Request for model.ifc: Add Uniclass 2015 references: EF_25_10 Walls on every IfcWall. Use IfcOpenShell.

First a look at what the model holds.

```python
import ifcopenshell

model = ifcopenshell.open("model.ifc")
print(model.schema)
print("classifications:", [c.Name for c in model.by_type("IfcClassification")])
for ifc_class in ("IfcDoor", "IfcRoof", "IfcStair", "IfcWall", "IfcWindow"):
    print(ifc_class, len(model.by_type(ifc_class)))
```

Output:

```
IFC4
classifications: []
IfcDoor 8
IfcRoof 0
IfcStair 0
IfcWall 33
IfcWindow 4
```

```python
import ifcopenshell
import ifcopenshell.api.classification

model = ifcopenshell.open("model.ifc")

system = ifcopenshell.api.classification.add_classification(model, classification="Uniclass 2015")

codes = {
    "IfcWall": ("EF_25_10", "Walls"),
}
for ifc_class, (code, name) in codes.items():
    products = model.by_type(ifc_class)
    ifcopenshell.api.classification.add_reference(
        model, products=products, classification=system, identification=code, name=name
    )
    print(code, len(products))

model.write("model_updated.ifc")
```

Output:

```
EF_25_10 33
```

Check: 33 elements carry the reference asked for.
